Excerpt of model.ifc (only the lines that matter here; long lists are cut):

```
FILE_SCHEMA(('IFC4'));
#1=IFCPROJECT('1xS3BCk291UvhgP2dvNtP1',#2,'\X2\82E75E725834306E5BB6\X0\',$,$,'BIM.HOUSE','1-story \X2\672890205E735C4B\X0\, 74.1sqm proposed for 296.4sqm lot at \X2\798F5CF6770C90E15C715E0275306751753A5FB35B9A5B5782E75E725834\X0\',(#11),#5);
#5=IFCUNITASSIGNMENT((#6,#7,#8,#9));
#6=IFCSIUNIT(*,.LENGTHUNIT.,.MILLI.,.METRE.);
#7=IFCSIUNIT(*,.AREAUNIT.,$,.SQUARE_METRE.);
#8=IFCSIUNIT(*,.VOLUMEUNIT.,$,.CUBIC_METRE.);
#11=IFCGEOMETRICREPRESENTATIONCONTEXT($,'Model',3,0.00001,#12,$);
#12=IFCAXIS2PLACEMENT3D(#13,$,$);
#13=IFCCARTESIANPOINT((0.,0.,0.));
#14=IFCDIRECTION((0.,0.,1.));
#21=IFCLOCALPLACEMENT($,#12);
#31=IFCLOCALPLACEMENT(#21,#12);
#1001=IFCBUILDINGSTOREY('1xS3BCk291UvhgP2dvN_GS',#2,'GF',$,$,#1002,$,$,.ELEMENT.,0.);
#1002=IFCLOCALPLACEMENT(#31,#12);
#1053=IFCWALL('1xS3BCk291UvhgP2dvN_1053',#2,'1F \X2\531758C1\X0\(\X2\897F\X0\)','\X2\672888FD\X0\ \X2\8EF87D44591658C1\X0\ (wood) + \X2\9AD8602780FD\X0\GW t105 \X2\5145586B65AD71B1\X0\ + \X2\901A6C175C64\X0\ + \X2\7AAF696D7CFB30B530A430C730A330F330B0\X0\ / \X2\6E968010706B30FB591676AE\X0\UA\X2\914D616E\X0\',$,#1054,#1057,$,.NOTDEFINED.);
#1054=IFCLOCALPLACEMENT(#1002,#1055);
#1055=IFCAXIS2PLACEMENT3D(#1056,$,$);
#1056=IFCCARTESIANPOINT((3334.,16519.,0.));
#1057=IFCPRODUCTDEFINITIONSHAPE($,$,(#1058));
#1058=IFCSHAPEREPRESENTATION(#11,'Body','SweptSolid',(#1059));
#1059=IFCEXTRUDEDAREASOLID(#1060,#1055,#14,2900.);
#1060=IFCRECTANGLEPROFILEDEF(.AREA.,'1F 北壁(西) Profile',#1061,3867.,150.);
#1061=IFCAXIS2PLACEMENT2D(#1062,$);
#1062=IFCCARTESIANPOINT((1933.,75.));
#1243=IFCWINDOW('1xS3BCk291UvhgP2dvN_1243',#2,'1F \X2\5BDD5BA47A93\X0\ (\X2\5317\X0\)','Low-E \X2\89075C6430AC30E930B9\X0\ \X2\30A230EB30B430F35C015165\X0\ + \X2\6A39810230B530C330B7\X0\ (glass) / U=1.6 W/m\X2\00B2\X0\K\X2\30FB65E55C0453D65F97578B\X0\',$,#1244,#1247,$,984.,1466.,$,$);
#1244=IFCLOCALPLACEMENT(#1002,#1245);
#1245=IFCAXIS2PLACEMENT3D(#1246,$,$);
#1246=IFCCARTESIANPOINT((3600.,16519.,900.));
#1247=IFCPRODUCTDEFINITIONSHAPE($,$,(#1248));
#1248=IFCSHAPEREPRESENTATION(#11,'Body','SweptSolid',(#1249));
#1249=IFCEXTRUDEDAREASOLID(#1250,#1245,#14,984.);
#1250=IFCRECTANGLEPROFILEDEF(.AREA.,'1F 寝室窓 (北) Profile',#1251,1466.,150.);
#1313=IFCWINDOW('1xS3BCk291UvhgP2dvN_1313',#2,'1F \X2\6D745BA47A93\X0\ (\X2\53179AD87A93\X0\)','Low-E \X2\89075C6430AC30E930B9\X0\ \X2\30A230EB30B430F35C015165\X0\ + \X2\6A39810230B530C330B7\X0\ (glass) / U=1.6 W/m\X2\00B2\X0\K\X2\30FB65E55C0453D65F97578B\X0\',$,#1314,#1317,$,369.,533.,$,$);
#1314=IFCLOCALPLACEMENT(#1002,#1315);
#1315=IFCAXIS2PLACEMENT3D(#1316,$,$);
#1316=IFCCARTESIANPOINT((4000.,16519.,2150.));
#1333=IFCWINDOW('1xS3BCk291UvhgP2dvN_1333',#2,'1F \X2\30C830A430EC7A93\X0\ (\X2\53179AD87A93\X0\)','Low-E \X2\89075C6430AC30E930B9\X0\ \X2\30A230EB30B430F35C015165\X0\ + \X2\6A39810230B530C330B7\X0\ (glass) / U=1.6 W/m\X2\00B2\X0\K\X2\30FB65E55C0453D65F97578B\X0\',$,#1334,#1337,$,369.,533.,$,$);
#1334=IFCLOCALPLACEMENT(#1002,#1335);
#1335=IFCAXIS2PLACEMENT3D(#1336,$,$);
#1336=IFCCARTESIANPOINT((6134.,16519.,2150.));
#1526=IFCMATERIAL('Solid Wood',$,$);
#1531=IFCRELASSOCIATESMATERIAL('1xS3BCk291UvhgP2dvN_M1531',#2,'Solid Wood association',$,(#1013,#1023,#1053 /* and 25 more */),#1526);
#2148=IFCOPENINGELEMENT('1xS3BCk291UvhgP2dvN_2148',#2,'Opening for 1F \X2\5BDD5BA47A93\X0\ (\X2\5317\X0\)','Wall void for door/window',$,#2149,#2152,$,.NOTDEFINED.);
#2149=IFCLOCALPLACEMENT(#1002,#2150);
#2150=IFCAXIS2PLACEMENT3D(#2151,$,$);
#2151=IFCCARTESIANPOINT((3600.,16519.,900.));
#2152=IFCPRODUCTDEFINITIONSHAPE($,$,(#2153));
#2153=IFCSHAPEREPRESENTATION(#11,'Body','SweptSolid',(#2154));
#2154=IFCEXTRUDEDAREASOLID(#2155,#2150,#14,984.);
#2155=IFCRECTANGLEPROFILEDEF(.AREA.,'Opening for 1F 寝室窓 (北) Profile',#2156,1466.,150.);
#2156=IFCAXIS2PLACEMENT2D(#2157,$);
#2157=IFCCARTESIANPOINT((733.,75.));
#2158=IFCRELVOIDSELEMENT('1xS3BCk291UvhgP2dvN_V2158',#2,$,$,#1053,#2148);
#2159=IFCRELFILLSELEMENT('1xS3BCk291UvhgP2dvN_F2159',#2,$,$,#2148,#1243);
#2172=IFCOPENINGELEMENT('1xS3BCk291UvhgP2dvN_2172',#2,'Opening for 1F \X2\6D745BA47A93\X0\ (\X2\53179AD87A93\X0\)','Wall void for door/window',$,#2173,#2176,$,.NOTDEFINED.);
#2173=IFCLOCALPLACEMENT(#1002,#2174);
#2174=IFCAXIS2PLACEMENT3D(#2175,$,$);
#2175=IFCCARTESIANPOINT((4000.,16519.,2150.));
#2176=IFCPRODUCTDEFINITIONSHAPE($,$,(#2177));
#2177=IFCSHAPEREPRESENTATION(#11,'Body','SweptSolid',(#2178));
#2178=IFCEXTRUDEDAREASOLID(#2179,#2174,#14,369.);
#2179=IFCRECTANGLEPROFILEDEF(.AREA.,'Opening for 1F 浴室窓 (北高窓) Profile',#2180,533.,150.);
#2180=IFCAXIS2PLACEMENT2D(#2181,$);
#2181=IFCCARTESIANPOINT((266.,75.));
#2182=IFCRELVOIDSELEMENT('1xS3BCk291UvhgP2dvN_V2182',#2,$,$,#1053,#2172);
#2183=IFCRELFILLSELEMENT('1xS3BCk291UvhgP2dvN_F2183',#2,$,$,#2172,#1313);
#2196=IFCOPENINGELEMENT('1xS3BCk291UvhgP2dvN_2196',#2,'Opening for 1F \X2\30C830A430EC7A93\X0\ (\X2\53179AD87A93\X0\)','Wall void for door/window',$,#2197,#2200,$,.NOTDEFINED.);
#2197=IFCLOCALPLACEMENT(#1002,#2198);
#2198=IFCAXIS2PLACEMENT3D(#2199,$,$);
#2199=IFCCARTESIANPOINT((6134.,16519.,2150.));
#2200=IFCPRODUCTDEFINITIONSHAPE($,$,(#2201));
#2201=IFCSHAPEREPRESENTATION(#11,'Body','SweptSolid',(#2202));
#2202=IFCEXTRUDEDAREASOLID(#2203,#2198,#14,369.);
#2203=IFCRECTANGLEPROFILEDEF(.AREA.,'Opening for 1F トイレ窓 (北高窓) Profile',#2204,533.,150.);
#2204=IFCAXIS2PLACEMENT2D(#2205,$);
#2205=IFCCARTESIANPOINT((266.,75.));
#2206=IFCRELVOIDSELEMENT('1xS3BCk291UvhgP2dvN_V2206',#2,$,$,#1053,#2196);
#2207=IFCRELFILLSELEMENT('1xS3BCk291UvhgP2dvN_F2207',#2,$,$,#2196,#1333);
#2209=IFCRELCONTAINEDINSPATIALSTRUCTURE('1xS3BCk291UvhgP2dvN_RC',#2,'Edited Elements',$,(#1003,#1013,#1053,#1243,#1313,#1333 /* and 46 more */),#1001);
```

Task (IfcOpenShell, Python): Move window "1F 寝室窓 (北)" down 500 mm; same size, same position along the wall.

```python
import numpy as np
import ifcopenshell
import ifcopenshell.api.geometry
import ifcopenshell.util.placement
import ifcopenshell.util.unit

model = ifcopenshell.open("model.ifc")
unit_scale = ifcopenshell.util.unit.calculate_unit_scale(model)

window = model.by_id(1243)
opening = window.FillsVoids[0].RelatingOpeningElement
dz = -0.5 / unit_scale

shift = np.array([0.0, 0.0, dz])
# The window is not placed relative to its opening, so move both.
for product in (opening, window):
    matrix = ifcopenshell.util.placement.get_local_placement(product.ObjectPlacement)
    matrix[:3, 3] += shift
    ifcopenshell.api.geometry.edit_object_placement(model, product=product, matrix=matrix, is_si=False)

print(f"moved by {dz * unit_scale:+.3f} m")

model.write("model_edited.ifc")
```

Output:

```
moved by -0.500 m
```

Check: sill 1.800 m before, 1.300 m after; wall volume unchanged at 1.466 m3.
